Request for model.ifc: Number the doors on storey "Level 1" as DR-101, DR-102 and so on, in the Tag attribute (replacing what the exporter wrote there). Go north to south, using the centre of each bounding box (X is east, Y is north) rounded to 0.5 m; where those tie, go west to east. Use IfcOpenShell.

First a look at what the model holds.

```python
import ifcopenshell
import ifcopenshell.util.element
import ifcopenshell.util.placement

model = ifcopenshell.open("model.ifc")
print(model.schema)
storey = next(s for s in model.by_type("IfcBuildingStorey") if s.Name == "Level 1")
doors = [e for e in ifcopenshell.util.element.get_decomposition(storey) if e.is_a("IfcDoor")]
for e in sorted(doors, key=lambda e: e.id()):
    origin = ifcopenshell.util.placement.get_local_placement(e.ObjectPlacement)[:3, 3]
    print(e.id(), e.Tag, e.Name, origin.round(2) + 0.0, sep=" | ")
```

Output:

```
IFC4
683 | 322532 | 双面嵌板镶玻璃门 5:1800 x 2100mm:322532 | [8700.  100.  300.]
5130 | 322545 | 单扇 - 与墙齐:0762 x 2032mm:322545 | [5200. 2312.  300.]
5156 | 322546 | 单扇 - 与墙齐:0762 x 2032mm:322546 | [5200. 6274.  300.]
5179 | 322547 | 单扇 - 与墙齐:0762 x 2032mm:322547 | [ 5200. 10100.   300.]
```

```python
import ifcopenshell
import ifcopenshell.geom
import ifcopenshell.util.element
import ifcopenshell.util.shape

model = ifcopenshell.open("model.ifc")
settings = ifcopenshell.geom.settings()
settings.set("use-world-coords", True)


def centre(element):
    shape = ifcopenshell.geom.create_shape(settings, element)
    return ifcopenshell.util.shape.get_bbox_centroid(shape.geometry)


storey = next(s for s in model.by_type("IfcBuildingStorey") if s.Name == "Level 1")
doors = [e for e in ifcopenshell.util.element.get_decomposition(storey) if e.is_a("IfcDoor")]

# Insertion points can sit at a corner or the storey origin, so sort by the geometry (in metres).
centres = {e: centre(e) for e in doors}
doors.sort(key=lambda e: (-round(centres[e][1] / 0.5), centres[e][0]))

for i, e in enumerate(doors, start=1):
    number = f"DR-1{i:02d}"
    e.Tag = number
    print(e.id(), number)

model.write("model_edited.ifc")
```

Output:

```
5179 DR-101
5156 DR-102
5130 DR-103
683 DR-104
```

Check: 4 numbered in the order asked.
